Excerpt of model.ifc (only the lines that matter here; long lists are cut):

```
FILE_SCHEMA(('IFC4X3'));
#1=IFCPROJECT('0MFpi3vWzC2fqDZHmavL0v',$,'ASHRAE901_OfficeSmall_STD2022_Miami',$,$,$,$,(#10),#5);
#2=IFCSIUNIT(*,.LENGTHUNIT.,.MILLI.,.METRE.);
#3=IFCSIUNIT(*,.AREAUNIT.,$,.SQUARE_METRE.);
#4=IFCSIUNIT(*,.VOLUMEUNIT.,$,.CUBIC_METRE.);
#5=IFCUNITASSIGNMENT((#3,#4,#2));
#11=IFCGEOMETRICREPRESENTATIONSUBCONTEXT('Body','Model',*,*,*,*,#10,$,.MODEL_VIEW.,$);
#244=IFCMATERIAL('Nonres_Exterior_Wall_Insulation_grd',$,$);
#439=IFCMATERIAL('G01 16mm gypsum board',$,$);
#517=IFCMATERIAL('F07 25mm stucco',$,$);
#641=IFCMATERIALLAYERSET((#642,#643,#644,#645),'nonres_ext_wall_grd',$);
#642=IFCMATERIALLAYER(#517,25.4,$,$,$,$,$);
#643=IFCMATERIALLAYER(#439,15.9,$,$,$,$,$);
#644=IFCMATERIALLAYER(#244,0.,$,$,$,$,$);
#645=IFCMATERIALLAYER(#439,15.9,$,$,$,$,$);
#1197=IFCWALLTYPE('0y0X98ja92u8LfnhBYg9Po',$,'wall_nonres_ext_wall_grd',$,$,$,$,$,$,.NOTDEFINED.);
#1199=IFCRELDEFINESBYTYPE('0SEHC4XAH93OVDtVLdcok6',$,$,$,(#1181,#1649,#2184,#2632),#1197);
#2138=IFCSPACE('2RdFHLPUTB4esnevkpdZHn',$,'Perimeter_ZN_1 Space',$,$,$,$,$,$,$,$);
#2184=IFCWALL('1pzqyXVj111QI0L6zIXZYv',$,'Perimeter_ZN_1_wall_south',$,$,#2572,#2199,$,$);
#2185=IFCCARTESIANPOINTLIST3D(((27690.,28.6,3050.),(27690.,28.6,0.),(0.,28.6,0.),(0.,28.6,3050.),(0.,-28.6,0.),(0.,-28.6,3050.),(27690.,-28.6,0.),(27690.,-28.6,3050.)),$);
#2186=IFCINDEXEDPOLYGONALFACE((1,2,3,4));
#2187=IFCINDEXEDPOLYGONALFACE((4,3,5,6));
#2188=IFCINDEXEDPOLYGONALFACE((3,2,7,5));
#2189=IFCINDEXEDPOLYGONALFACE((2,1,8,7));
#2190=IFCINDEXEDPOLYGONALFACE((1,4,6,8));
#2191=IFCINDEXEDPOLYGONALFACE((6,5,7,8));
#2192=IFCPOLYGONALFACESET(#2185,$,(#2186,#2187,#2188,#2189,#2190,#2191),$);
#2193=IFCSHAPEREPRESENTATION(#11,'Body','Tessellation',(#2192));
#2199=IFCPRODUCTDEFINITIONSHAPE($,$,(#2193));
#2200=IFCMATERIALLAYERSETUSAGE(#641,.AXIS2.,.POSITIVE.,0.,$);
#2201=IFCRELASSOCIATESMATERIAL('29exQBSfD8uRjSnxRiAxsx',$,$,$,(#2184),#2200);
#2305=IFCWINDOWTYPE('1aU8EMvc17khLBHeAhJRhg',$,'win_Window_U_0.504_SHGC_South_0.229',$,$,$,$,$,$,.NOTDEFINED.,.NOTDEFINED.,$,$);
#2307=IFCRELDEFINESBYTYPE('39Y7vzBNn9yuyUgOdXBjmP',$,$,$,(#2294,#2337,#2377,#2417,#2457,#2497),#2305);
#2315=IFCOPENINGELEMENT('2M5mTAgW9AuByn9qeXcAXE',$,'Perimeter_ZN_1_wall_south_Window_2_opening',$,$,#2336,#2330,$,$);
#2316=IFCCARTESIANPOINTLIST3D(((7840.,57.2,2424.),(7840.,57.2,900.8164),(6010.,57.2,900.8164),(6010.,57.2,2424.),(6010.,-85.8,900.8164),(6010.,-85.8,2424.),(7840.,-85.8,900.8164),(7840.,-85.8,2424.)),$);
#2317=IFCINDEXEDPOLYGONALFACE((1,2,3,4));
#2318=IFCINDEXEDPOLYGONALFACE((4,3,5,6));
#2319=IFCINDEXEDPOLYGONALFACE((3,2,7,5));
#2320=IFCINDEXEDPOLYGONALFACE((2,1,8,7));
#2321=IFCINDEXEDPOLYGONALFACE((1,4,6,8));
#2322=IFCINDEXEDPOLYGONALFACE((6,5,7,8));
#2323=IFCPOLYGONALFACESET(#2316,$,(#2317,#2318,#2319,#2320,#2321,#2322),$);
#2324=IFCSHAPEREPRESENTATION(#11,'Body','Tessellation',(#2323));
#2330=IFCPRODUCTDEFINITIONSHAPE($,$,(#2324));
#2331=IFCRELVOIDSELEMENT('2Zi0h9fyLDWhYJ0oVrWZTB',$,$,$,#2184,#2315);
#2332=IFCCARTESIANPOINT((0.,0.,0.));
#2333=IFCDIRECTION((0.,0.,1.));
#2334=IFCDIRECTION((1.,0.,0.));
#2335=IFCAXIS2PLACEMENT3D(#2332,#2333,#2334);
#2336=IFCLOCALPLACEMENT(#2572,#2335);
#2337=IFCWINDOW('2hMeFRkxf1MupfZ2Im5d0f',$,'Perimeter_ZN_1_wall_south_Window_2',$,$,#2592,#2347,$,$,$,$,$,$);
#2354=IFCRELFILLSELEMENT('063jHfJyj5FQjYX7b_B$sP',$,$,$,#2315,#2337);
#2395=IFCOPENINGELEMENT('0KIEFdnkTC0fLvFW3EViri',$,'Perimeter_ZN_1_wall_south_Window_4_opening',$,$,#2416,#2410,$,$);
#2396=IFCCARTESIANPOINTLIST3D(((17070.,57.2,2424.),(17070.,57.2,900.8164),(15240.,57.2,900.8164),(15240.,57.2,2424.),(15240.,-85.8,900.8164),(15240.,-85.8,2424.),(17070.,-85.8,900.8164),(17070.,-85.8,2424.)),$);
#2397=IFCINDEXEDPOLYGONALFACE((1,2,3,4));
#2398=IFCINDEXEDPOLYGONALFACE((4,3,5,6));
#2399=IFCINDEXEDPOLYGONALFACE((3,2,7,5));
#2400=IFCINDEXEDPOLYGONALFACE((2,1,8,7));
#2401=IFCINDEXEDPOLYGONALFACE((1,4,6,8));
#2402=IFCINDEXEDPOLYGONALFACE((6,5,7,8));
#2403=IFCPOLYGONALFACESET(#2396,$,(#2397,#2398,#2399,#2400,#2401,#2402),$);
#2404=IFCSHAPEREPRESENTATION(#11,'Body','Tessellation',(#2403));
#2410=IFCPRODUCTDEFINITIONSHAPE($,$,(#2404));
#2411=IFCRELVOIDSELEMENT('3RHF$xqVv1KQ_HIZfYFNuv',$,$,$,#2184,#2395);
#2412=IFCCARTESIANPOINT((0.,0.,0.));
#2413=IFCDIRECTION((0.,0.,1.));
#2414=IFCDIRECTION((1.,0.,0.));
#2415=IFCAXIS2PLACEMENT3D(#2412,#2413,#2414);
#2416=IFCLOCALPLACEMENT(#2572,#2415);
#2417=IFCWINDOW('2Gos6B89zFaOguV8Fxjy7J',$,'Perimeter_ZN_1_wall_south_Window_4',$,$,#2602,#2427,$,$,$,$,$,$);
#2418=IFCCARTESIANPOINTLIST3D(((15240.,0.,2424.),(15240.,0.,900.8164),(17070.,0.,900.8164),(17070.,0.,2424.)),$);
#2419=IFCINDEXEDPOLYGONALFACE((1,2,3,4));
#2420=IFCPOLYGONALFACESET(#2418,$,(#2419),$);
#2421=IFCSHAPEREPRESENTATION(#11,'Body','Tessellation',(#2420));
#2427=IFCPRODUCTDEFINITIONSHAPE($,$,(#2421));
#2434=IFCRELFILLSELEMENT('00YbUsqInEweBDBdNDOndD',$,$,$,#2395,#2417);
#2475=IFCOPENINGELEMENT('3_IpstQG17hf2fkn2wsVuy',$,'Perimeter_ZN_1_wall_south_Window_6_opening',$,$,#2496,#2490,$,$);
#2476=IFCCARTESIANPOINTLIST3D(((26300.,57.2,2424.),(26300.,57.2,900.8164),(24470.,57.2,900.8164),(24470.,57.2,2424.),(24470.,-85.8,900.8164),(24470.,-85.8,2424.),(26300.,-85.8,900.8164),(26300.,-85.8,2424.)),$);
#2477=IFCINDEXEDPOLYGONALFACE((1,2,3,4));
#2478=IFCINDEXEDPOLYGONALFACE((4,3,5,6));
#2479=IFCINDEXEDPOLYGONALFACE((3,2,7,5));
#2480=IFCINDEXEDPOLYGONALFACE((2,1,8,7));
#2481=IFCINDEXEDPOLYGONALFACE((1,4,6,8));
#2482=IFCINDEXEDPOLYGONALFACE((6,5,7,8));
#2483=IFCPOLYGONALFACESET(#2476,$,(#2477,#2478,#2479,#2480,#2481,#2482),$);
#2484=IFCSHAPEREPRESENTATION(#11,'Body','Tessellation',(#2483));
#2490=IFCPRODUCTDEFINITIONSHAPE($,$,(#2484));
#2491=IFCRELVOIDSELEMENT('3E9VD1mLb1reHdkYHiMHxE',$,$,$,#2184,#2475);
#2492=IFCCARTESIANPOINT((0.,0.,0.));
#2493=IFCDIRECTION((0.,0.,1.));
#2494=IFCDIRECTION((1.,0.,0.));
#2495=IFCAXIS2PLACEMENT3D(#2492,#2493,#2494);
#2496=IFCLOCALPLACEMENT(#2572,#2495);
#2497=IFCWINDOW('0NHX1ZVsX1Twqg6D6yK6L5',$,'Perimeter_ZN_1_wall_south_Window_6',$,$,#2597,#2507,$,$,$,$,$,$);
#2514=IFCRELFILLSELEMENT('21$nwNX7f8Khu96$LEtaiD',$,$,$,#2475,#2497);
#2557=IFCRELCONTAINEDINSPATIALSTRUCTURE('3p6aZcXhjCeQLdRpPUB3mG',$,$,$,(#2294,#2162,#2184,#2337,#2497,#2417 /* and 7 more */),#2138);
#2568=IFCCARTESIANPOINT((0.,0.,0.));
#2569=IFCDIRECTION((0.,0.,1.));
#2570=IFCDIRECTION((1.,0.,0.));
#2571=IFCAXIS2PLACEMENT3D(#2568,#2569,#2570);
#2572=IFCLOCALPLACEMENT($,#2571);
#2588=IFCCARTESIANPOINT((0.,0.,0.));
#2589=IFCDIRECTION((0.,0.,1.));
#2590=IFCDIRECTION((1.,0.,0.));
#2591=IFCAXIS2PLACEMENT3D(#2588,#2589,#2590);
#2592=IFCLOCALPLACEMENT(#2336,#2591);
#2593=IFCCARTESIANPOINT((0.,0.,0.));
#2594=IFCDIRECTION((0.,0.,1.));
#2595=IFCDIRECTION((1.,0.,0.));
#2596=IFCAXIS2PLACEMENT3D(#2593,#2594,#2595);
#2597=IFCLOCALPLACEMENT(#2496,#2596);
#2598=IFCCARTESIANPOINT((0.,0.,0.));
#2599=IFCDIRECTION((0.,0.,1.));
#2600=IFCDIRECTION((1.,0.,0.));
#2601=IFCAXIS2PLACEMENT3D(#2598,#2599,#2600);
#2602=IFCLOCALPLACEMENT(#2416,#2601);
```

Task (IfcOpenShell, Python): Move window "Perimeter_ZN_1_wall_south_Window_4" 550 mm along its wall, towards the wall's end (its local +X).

```python
import ifcopenshell
import ifcopenshell.api.geometry
import ifcopenshell.util.placement

model = ifcopenshell.open("model.ifc")

window = model.by_guid("2Gos6B89zFaOguV8Fxjy7J")
opening = window.FillsVoids[0].RelatingOpeningElement
wall = opening.VoidsElements[0].RelatingBuildingElement

wall_matrix = ifcopenshell.util.placement.get_local_placement(wall.ObjectPlacement)
shift = wall_matrix[:3, 0] * 550.0
before = ifcopenshell.util.placement.get_local_placement(window.ObjectPlacement)[:3, 3].copy()

# The window is placed relative to its opening, so it follows when the opening moves.
matrix = ifcopenshell.util.placement.get_local_placement(opening.ObjectPlacement)
matrix[:3, 3] += shift
ifcopenshell.api.geometry.edit_object_placement(
    model, product=opening, matrix=matrix, is_si=False, should_transform_children=True
)

after = ifcopenshell.util.placement.get_local_placement(window.ObjectPlacement)[:3, 3]
print("window moved by", (after - before).round(3) + 0.0)

model.write("model_edited.ifc")
```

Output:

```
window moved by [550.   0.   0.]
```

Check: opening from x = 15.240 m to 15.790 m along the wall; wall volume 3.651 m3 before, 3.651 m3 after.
